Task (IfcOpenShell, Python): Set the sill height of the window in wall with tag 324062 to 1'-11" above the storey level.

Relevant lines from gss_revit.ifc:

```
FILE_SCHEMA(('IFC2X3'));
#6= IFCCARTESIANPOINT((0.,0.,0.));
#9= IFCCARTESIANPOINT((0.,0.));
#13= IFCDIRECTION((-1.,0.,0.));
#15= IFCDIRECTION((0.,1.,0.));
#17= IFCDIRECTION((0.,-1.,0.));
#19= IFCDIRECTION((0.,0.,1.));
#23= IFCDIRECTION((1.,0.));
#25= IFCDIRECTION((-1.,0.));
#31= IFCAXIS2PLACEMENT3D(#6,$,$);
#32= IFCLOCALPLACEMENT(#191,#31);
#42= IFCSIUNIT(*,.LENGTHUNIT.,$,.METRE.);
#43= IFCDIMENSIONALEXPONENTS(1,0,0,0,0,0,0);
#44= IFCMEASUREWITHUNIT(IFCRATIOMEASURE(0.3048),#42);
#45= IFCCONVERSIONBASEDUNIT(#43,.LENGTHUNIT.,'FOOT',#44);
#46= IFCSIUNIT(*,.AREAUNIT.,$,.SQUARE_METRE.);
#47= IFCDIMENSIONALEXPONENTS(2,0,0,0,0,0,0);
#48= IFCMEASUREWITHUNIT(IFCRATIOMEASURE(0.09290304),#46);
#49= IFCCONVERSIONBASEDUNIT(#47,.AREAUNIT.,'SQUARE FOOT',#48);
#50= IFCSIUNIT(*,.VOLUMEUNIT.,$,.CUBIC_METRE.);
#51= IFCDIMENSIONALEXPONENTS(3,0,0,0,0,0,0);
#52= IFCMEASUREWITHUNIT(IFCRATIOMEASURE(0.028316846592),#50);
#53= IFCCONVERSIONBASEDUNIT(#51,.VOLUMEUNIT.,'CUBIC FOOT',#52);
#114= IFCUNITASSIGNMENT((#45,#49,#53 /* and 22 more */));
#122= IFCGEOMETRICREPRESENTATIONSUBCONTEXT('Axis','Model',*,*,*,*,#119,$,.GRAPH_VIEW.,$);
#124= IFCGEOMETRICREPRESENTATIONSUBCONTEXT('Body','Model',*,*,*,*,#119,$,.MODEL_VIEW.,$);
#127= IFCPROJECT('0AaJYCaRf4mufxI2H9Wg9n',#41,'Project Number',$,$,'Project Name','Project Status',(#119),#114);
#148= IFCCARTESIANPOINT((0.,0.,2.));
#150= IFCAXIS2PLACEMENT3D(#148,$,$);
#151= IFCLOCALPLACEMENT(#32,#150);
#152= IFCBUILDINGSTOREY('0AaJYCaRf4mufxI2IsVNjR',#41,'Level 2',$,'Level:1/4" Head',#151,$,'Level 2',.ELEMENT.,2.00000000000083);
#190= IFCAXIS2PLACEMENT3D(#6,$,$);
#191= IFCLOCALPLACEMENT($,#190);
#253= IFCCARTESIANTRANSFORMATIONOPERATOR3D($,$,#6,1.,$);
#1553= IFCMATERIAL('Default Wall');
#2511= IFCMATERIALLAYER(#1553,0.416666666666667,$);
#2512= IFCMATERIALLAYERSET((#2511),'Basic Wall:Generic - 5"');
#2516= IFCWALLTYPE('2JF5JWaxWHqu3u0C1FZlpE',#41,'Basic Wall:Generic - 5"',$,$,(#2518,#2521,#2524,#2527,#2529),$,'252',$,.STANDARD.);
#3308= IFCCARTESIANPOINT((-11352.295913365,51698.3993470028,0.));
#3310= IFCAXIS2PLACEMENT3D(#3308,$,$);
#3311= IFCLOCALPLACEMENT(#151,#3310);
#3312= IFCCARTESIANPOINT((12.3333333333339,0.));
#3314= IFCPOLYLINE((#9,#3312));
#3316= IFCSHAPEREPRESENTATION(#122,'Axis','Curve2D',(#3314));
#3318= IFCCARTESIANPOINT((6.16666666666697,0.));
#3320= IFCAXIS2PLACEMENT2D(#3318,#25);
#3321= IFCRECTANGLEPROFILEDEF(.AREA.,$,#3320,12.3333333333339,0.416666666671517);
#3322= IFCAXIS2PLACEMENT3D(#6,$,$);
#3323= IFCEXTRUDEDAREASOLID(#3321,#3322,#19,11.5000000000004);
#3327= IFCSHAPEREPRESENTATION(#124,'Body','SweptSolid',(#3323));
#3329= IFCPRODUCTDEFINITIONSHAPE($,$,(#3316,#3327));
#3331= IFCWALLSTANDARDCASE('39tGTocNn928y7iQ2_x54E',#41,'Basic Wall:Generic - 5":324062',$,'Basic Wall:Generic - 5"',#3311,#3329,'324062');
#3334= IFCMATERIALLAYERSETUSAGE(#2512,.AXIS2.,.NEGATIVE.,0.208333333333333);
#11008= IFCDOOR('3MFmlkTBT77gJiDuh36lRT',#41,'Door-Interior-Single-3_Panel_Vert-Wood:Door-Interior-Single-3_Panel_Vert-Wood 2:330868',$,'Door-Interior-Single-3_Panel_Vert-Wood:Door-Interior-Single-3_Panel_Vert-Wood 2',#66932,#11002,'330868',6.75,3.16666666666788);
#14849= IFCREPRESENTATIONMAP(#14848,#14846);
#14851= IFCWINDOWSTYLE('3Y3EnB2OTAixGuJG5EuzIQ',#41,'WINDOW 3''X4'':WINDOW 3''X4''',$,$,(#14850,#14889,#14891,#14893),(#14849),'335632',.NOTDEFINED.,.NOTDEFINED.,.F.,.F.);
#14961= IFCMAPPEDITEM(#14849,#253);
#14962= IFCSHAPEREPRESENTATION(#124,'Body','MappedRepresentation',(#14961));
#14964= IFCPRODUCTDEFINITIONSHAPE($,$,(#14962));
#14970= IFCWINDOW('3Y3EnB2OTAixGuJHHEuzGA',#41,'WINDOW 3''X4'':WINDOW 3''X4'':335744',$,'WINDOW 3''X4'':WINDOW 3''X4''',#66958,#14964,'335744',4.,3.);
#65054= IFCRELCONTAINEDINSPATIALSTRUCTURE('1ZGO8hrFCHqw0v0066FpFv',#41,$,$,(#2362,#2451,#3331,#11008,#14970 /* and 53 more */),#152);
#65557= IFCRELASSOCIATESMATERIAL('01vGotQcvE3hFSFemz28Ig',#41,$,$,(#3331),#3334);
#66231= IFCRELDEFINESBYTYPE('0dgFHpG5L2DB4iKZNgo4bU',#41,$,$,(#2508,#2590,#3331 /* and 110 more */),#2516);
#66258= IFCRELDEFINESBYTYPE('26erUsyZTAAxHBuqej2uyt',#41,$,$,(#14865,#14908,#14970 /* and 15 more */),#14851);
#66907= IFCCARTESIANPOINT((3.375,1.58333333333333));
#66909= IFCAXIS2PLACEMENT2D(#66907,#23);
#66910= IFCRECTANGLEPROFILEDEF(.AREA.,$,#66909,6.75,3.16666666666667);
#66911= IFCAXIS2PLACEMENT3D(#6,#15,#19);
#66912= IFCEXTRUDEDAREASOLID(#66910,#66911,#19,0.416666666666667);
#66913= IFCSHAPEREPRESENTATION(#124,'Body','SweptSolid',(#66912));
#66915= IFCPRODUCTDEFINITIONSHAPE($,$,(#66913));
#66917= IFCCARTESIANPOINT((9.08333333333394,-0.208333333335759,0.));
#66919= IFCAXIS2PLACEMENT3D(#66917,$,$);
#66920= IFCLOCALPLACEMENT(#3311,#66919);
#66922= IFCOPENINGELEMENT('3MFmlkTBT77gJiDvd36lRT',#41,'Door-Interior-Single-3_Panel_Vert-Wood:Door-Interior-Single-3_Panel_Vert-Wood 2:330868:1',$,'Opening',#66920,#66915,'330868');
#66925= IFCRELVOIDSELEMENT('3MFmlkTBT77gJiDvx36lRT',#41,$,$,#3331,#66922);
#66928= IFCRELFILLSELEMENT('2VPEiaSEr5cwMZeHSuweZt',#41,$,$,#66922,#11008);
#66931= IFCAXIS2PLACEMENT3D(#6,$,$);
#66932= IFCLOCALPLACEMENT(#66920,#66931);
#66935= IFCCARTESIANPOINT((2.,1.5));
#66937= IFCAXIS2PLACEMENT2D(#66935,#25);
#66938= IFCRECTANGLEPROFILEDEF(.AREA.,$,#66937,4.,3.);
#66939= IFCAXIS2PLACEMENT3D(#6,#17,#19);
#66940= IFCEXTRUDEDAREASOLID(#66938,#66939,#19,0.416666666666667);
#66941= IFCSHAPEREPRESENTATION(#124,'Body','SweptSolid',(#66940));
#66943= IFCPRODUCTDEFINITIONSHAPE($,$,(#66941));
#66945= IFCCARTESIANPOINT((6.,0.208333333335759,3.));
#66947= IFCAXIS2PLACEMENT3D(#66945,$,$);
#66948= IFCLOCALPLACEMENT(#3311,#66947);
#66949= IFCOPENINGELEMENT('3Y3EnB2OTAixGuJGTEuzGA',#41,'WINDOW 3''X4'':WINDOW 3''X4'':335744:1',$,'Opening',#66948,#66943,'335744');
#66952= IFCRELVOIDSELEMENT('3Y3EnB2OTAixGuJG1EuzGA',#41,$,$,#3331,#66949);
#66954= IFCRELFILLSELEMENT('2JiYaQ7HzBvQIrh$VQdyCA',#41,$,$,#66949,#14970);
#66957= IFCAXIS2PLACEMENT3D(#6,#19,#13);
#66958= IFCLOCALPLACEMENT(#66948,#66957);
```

```python
import numpy as np
import ifcopenshell
import ifcopenshell.api.geometry
import ifcopenshell.geom
import ifcopenshell.util.element
import ifcopenshell.util.placement
import ifcopenshell.util.shape
import ifcopenshell.util.unit

model = ifcopenshell.open("gss_revit.ifc")
unit_scale = ifcopenshell.util.unit.calculate_unit_scale(model)

window = model.by_guid("3Y3EnB2OTAixGuJHHEuzGA")
opening = window.FillsVoids[0].RelatingOpeningElement
storey = ifcopenshell.util.element.get_container(window, ifc_class="IfcBuildingStorey")
level = ifcopenshell.util.placement.get_local_placement(storey.ObjectPlacement)[2, 3]

# The opening's origin need not be at the sill, so measure its lowest point.
shape = ifcopenshell.geom.create_shape(ifcopenshell.geom.settings(), opening)
bottom = ifcopenshell.util.shape.get_shape_bottom_elevation(shape, shape.geometry) / unit_scale
dz = level + 23 * 0.0254 / unit_scale - bottom

shift = np.array([0.0, 0.0, dz])
# The window is placed relative to its opening, so it follows when the opening moves.
matrix = ifcopenshell.util.placement.get_local_placement(opening.ObjectPlacement)
matrix[:3, 3] += shift
ifcopenshell.api.geometry.edit_object_placement(
    model, product=opening, matrix=matrix, is_si=False, should_transform_children=True
)

print(f"moved by {dz * unit_scale:+.3f} m")

model.write("gss_revit_v2.ifc")
```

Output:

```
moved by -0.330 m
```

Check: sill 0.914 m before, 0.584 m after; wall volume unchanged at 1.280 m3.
